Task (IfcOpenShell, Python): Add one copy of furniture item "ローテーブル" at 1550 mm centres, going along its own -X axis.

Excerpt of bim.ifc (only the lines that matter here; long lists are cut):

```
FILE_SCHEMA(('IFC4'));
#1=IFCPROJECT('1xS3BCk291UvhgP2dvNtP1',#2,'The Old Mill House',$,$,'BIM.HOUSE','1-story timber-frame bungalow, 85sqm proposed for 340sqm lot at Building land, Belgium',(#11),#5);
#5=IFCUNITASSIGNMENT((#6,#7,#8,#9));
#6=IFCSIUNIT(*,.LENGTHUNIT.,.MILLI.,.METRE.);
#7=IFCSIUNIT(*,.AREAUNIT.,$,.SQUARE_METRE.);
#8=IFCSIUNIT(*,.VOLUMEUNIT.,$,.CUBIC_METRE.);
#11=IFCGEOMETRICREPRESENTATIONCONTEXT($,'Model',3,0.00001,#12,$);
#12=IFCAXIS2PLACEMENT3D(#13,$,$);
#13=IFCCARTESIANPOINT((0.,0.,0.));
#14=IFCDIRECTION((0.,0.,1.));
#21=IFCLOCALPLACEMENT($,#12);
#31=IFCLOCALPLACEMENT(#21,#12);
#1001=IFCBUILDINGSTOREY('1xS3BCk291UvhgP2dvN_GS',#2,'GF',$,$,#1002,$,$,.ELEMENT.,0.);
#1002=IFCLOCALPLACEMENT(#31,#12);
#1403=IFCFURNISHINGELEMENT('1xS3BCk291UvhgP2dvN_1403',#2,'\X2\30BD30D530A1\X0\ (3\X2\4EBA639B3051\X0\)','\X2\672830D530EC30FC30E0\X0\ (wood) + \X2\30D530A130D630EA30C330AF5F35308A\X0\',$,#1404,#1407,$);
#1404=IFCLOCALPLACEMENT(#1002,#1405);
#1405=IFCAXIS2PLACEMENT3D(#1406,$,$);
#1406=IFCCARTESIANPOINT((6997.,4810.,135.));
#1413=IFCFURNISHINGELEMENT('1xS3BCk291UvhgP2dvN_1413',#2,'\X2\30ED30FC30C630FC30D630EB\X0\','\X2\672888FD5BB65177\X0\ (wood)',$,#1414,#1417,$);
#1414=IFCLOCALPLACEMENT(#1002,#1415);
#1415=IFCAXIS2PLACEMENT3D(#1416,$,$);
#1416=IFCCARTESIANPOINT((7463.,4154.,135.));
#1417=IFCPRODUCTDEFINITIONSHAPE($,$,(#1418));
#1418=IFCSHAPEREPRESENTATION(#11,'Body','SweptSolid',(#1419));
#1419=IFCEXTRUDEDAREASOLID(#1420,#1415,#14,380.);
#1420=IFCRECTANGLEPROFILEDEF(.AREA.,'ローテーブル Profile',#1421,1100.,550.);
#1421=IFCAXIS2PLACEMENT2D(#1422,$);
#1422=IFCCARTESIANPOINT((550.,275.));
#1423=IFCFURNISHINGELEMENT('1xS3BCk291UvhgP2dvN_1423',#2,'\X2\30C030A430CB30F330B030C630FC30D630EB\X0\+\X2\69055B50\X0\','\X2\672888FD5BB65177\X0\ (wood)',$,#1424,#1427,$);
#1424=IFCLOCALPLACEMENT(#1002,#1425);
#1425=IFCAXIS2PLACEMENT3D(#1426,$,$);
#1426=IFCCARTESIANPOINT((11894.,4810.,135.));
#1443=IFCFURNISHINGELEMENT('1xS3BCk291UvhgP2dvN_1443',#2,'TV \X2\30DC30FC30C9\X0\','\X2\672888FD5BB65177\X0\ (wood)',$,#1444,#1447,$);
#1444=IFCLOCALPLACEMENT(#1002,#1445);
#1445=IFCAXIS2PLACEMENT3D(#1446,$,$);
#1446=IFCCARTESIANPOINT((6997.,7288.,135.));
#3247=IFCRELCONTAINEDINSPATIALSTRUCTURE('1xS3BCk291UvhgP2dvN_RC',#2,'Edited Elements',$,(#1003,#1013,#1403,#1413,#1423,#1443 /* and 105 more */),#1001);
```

```python
import ifcopenshell
import ifcopenshell.api.geometry
import ifcopenshell.api.root
import ifcopenshell.util.element
import ifcopenshell.util.placement

model = ifcopenshell.open("bim.ifc")


def reuse_history(source, copy):
    """copy_class also copies each property set's owner history, people and application; keep the originals."""
    for rel in copy.IsDefinedBy:
        if rel.is_a("IfcRelDefinesByProperties") and (history := rel.RelatingPropertyDefinition.OwnerHistory):
            rel.RelatingPropertyDefinition.OwnerHistory = source.OwnerHistory
            ifcopenshell.util.element.remove_deep2(model, history)


source = model.by_guid("1xS3BCk291UvhgP2dvN_1413")
base = ifcopenshell.util.placement.get_local_placement(source.ObjectPlacement)
step = -base[:3, 0] * 1550.0

for i in range(1, 2):
    copy = ifcopenshell.api.root.copy_class(model, product=source)
    copy.Representation = ifcopenshell.util.element.copy_deep(
        model, source.Representation, exclude=["IfcGeometricRepresentationContext", "IfcRepresentationMap"]
    )
    reuse_history(source, copy)
    matrix = base.copy()
    matrix[:3, 3] += i * step
    print("added at", matrix[:3, 3].round(3) + 0.0)
    ifcopenshell.api.geometry.edit_object_placement(model, product=copy, matrix=matrix, is_si=False)

model.write("bim_updated.ifc")
```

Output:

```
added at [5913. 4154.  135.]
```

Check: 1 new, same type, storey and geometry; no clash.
